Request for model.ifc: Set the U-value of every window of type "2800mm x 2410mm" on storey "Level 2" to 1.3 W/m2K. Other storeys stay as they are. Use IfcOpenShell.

First a look at what the model holds.

```python
import ifcopenshell
import ifcopenshell.util.element

model = ifcopenshell.open("model.ifc")
print(model.schema)
storey = next(s for s in model.by_type("IfcBuildingStorey") if s.Name == "Level 2")
windows = [e for e in ifcopenshell.util.element.get_decomposition(storey) if e.is_a("IfcWindow")]
seen = {}
for e in windows:
    element_type = ifcopenshell.util.element.get_type(e)
    key = (element_type.Name if element_type != e and element_type else None, ifcopenshell.util.element.get_pset(e, "Pset_WindowCommon", "ThermalTransmittance"))
    seen[key] = seen.get(key, 0) + 1
for (name, value), count in sorted(seen.items(), key=str):
    print(count, "x", name, "|", value)
```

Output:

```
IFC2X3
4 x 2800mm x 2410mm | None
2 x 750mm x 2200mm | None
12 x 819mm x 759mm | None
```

```python
import ifcopenshell
import ifcopenshell.api.pset
import ifcopenshell.util.element

model = ifcopenshell.open("model.ifc")

storey = next(s for s in model.by_type("IfcBuildingStorey") if s.Name == "Level 2")
windows = [e for e in ifcopenshell.util.element.get_decomposition(storey) if e.is_a("IfcWindow")]

count = 0
for e in windows:
    element_type = ifcopenshell.util.element.get_type(e)
    if element_type in (None, e) or element_type.Name != "2800mm x 2410mm":
        continue
    # add_pset returns the element's existing set when there is one.
    pset = ifcopenshell.api.pset.add_pset(model, product=e, name="Pset_WindowCommon")
    ifcopenshell.api.pset.edit_pset(model, pset=pset, properties={"ThermalTransmittance": 1.3})
    count += 1

print(count, "windows updated")

model.write("model_rev.ifc")
```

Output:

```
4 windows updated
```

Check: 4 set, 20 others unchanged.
